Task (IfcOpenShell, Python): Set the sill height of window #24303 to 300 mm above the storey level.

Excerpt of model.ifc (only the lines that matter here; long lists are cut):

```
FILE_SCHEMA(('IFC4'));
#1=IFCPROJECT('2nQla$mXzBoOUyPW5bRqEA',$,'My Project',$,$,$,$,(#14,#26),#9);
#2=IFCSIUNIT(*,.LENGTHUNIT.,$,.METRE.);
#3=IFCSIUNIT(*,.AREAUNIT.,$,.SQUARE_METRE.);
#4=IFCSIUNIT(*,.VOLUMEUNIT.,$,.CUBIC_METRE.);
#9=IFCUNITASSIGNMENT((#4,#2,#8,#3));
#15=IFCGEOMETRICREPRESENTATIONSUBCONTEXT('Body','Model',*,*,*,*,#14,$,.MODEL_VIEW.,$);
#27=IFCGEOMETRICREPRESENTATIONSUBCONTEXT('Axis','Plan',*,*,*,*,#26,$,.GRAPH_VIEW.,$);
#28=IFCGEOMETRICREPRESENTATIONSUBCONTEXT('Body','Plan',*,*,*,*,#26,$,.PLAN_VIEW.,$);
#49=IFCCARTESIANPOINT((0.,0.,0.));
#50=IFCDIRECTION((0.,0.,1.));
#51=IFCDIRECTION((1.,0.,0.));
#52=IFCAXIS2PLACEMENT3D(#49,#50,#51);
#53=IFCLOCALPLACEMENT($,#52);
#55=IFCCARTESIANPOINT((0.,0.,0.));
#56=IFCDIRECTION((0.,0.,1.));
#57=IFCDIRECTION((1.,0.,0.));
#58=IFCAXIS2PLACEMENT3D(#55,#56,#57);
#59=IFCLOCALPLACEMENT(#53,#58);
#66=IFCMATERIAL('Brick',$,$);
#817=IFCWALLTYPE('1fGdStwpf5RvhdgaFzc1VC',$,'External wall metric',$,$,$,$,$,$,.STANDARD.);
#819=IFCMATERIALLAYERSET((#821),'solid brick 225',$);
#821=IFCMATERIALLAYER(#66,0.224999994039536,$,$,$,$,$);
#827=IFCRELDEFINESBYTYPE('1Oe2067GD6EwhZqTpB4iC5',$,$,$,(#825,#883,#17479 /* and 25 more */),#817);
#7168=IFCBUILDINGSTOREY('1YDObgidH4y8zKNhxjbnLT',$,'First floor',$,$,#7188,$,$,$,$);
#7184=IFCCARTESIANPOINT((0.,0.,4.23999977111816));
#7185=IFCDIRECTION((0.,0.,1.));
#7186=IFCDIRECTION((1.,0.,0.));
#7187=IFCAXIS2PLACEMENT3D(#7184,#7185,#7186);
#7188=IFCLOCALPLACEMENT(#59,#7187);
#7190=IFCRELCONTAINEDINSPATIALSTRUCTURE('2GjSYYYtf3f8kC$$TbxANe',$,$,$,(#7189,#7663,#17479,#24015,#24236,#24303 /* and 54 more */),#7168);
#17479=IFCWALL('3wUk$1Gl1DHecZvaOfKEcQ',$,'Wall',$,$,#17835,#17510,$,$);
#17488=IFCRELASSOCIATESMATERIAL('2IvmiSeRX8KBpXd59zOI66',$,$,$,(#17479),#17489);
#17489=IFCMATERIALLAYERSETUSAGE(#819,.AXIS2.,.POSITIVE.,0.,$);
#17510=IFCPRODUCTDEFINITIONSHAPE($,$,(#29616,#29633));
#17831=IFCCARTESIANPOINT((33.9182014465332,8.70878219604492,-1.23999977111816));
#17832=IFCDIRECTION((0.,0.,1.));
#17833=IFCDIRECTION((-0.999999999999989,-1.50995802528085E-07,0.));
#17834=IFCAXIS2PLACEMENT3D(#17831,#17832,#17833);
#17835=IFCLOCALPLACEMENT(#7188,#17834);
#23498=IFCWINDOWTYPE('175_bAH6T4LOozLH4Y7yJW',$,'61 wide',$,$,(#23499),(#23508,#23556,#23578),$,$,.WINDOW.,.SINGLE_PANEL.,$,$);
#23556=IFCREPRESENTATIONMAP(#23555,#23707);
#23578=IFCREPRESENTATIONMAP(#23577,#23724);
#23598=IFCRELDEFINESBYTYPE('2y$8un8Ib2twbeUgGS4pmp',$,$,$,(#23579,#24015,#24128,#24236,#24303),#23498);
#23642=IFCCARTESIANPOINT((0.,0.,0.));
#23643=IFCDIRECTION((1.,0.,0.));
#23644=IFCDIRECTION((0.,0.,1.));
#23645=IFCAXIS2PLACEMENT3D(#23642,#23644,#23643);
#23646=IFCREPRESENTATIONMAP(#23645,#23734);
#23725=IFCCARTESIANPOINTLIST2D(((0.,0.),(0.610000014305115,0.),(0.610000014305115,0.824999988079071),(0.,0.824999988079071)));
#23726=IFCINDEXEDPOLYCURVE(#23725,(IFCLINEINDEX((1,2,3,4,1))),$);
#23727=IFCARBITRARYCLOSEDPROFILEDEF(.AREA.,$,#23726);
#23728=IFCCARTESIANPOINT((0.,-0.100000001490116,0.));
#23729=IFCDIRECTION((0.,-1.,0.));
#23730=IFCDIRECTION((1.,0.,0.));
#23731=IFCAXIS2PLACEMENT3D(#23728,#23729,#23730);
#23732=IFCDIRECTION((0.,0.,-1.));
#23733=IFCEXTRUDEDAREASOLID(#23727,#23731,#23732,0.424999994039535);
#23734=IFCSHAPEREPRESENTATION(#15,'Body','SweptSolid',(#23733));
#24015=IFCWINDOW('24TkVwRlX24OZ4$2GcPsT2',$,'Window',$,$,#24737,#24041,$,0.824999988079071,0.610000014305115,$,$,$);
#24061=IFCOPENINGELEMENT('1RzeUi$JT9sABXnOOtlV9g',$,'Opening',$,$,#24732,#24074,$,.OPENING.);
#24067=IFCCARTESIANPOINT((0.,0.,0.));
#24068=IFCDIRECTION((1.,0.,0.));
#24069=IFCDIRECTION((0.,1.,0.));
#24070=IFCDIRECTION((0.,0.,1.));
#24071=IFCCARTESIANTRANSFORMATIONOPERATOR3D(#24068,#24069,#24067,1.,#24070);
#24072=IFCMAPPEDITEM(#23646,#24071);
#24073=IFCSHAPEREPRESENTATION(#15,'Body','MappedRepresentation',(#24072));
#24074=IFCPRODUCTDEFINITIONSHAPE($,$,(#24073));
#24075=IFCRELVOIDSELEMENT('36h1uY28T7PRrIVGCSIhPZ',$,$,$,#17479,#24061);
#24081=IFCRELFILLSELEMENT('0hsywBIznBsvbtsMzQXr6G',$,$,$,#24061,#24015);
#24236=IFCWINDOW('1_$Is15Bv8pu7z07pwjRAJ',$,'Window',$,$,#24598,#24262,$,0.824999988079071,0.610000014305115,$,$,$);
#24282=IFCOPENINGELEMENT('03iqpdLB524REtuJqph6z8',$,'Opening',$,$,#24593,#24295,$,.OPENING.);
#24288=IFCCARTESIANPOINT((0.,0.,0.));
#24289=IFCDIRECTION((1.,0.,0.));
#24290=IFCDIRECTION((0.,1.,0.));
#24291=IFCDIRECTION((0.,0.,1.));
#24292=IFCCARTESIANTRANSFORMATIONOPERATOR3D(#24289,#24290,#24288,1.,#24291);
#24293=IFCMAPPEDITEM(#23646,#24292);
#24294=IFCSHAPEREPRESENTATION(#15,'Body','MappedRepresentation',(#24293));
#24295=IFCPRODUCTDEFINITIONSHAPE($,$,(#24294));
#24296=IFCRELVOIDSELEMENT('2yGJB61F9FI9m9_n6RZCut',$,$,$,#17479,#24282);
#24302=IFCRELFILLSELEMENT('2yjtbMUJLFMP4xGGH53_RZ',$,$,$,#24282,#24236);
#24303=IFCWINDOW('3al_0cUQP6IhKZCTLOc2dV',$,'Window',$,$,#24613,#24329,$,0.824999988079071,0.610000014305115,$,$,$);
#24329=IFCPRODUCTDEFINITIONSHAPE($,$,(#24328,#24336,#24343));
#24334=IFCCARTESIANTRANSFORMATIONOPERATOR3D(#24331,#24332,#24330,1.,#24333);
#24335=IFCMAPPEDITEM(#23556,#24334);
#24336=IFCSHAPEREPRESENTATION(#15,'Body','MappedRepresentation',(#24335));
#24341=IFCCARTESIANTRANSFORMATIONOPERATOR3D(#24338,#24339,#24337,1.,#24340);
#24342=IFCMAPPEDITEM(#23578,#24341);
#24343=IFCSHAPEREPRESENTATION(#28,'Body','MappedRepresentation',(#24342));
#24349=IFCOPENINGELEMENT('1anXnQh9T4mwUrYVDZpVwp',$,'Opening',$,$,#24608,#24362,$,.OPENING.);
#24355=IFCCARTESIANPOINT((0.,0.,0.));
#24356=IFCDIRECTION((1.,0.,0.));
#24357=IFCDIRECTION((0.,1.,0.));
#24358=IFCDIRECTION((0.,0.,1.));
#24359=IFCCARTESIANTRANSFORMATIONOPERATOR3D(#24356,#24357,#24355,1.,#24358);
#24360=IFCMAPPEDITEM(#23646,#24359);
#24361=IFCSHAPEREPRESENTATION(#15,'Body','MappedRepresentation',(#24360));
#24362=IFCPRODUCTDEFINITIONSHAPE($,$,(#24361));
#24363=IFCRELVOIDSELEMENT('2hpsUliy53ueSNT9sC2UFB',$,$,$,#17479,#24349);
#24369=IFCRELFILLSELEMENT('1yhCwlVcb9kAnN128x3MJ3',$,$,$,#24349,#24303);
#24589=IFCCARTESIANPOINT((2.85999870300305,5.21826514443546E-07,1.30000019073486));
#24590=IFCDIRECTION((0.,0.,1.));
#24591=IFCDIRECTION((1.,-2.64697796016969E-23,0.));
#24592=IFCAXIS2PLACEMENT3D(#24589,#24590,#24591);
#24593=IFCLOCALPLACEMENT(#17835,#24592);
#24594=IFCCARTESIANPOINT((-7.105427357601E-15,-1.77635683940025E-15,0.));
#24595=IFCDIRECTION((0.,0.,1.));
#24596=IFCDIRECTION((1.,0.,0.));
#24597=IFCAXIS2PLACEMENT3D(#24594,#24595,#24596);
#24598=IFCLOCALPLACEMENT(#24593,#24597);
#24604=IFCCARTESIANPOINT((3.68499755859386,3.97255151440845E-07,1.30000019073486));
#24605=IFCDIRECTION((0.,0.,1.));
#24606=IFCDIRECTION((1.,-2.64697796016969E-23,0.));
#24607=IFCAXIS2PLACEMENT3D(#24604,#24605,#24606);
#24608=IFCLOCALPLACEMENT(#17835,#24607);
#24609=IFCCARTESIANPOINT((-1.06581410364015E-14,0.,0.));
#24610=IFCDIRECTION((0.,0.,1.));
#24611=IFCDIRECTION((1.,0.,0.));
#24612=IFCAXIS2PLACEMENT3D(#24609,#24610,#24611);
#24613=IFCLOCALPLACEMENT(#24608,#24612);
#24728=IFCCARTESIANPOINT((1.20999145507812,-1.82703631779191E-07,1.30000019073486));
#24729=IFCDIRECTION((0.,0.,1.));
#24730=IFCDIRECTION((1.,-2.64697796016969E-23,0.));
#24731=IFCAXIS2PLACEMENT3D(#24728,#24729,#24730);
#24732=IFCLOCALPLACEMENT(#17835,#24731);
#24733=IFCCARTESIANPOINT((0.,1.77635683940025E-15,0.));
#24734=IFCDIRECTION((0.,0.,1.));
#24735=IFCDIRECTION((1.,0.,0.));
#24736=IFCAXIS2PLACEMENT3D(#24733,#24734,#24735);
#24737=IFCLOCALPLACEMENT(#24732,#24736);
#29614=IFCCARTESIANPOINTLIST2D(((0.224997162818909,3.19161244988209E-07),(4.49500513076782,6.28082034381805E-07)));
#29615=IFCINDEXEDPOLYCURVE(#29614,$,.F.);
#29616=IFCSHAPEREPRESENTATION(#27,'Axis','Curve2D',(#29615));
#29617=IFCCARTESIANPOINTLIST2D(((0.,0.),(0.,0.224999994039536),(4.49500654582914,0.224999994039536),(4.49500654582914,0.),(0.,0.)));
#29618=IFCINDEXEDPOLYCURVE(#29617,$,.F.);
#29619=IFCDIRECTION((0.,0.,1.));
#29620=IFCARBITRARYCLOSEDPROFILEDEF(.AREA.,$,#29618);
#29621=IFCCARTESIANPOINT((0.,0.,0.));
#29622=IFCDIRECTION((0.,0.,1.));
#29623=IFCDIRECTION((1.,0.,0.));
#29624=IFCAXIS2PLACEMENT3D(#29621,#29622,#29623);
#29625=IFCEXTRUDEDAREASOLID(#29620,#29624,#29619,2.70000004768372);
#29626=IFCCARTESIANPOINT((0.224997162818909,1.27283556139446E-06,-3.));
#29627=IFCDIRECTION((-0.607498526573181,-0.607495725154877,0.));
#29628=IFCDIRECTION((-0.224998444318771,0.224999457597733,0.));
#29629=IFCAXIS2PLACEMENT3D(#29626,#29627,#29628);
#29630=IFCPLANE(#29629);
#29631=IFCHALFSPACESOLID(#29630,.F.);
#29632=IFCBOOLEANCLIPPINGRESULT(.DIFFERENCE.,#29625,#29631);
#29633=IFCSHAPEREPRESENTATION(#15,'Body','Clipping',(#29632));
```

```python
import numpy as np
import ifcopenshell
import ifcopenshell.api.geometry
import ifcopenshell.geom
import ifcopenshell.util.element
import ifcopenshell.util.placement
import ifcopenshell.util.shape
import ifcopenshell.util.unit

model = ifcopenshell.open("model.ifc")
unit_scale = ifcopenshell.util.unit.calculate_unit_scale(model)

window = model.by_guid("3al_0cUQP6IhKZCTLOc2dV")
opening = window.FillsVoids[0].RelatingOpeningElement
storey = ifcopenshell.util.element.get_container(window, ifc_class="IfcBuildingStorey")
level = ifcopenshell.util.placement.get_local_placement(storey.ObjectPlacement)[2, 3]

# The opening's origin need not be at the sill, so measure its lowest point.
shape = ifcopenshell.geom.create_shape(ifcopenshell.geom.settings(), opening)
bottom = ifcopenshell.util.shape.get_shape_bottom_elevation(shape, shape.geometry) / unit_scale
dz = level + 0.3 / unit_scale - bottom

shift = np.array([0.0, 0.0, dz])
# The window is placed relative to its opening, so it follows when the opening moves.
matrix = ifcopenshell.util.placement.get_local_placement(opening.ObjectPlacement)
matrix[:3, 3] += shift
ifcopenshell.api.geometry.edit_object_placement(
    model, product=opening, matrix=matrix, is_si=False, should_transform_children=True
)

print(f"moved by {dz * unit_scale:+.3f} m")

model.write("model-out.ifc")
```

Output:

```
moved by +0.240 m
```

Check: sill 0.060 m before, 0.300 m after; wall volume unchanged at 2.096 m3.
